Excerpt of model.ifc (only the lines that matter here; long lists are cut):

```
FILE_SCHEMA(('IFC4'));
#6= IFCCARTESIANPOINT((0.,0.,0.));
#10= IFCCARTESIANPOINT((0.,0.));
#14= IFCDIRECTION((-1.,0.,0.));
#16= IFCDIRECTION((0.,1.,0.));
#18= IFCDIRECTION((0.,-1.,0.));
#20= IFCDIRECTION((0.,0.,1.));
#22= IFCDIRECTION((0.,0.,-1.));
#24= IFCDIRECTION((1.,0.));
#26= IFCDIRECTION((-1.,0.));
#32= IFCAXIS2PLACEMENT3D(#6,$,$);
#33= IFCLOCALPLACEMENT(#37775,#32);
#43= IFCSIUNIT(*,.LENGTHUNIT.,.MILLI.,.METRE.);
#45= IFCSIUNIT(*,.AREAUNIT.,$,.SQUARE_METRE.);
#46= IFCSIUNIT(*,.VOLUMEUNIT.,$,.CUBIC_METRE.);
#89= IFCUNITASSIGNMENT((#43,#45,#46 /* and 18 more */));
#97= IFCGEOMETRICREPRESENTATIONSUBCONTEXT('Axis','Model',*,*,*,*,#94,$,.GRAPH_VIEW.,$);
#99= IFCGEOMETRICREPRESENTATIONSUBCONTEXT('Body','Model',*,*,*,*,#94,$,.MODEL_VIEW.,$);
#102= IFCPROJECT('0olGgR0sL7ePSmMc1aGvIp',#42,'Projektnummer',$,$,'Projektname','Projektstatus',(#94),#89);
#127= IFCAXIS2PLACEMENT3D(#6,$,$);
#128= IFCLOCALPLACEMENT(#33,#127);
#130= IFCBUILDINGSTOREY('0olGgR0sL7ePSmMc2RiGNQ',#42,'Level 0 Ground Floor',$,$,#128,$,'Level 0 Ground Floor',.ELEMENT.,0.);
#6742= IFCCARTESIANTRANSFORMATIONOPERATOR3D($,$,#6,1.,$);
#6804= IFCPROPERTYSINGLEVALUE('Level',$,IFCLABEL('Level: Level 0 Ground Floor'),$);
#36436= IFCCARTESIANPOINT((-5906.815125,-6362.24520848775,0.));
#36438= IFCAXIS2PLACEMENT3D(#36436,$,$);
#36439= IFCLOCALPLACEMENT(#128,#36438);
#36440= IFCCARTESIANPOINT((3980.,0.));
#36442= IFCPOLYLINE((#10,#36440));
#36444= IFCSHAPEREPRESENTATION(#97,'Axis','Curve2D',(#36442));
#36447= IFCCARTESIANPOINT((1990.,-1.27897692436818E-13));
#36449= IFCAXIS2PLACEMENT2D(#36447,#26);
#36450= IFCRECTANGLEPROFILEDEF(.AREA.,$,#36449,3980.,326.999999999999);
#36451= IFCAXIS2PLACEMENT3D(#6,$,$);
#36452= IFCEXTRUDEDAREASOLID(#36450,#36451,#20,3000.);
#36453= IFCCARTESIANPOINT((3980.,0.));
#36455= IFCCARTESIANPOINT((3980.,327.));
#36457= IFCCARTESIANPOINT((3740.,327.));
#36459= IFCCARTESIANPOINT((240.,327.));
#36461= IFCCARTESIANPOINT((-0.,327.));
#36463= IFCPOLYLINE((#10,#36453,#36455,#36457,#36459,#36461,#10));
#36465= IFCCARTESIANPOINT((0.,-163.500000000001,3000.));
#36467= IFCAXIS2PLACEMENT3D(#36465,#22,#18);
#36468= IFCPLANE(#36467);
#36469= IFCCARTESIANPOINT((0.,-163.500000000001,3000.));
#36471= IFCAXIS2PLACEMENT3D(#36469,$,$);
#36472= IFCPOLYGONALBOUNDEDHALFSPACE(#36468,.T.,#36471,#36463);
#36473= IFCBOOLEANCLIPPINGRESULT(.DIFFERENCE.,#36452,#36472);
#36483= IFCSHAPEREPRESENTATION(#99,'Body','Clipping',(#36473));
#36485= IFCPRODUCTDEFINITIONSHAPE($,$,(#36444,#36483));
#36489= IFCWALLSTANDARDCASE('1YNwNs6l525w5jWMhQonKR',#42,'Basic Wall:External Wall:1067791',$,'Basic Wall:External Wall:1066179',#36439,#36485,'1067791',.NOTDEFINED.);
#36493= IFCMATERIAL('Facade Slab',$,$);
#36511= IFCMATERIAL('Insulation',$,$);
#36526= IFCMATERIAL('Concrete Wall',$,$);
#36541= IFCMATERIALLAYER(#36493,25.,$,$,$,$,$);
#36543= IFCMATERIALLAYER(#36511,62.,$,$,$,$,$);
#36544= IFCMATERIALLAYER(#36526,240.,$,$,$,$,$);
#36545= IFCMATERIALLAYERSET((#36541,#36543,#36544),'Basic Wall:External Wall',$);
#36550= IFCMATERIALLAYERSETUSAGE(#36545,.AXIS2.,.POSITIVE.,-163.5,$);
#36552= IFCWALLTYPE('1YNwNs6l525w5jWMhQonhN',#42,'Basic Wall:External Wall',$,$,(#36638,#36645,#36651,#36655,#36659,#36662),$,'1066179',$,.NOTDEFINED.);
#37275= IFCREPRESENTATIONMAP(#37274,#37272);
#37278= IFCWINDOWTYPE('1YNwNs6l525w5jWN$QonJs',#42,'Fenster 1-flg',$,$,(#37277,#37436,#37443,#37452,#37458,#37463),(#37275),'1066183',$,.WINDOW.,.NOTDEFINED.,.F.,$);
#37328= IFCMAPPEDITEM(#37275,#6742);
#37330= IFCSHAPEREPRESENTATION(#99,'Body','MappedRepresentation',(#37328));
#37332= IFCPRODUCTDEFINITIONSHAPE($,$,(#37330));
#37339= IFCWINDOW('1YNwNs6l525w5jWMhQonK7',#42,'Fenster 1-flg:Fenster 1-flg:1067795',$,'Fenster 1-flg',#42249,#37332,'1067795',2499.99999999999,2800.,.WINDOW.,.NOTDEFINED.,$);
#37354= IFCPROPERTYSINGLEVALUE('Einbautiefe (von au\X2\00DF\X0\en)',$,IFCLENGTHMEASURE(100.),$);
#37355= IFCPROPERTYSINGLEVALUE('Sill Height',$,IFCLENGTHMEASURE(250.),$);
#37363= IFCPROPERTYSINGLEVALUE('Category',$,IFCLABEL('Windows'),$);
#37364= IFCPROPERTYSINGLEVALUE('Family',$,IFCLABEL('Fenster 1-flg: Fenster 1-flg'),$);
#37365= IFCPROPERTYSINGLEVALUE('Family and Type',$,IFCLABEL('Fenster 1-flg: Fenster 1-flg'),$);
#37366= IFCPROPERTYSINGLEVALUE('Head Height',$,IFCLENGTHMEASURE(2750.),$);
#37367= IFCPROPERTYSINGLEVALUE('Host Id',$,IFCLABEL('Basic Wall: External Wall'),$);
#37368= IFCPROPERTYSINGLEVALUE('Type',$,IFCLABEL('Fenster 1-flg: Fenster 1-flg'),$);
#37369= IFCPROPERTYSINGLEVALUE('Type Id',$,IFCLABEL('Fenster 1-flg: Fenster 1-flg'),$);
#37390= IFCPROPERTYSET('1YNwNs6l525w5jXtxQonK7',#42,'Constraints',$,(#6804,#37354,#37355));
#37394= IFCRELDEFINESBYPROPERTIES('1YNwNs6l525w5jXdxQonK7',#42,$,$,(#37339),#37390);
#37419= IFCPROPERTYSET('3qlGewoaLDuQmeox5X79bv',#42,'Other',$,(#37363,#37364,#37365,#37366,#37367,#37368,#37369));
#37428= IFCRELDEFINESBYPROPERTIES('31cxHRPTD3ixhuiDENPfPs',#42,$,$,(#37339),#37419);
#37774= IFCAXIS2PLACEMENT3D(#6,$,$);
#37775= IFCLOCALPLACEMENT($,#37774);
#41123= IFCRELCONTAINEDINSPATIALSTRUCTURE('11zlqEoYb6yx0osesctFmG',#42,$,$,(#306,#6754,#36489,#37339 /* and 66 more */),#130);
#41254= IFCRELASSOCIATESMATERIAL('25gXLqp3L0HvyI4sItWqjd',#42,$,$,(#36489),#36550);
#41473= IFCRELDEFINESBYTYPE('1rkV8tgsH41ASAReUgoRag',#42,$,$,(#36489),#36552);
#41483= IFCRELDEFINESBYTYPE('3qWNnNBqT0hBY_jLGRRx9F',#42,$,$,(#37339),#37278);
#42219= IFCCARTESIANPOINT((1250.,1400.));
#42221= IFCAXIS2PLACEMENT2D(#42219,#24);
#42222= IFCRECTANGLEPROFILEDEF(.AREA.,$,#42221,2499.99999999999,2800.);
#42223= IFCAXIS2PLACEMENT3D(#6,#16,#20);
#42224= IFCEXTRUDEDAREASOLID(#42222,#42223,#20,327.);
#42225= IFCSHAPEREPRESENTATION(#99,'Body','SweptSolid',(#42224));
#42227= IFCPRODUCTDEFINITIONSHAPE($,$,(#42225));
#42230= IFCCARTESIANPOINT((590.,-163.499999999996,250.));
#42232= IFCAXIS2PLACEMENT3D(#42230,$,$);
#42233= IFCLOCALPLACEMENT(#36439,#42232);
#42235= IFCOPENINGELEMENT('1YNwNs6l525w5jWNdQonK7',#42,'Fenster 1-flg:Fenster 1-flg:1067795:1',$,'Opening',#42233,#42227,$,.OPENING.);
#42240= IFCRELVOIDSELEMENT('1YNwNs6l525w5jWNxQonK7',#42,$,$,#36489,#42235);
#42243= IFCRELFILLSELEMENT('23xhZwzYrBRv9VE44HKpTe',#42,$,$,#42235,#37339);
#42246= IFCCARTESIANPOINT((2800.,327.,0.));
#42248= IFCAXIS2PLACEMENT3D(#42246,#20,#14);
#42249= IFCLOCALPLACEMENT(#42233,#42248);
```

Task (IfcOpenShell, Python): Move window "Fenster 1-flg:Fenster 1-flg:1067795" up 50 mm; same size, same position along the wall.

```python
import numpy as np
import ifcopenshell
import ifcopenshell.api.geometry
import ifcopenshell.api.pset
import ifcopenshell.util.element
import ifcopenshell.util.placement
import ifcopenshell.util.unit

model = ifcopenshell.open("model.ifc")
unit_scale = ifcopenshell.util.unit.calculate_unit_scale(model)

window = model.by_guid("1YNwNs6l525w5jWMhQonK7")
opening = window.FillsVoids[0].RelatingOpeningElement
dz = 0.05 / unit_scale

shift = np.array([0.0, 0.0, dz])
# The window is placed relative to its opening, so it follows when the opening moves.
matrix = ifcopenshell.util.placement.get_local_placement(opening.ObjectPlacement)
matrix[:3, 3] += shift
ifcopenshell.api.geometry.edit_object_placement(
    model, product=opening, matrix=matrix, is_si=False, should_transform_children=True
)

# Keep the stored heights in step.
pset = model.by_id(ifcopenshell.util.element.get_pset(window, "Constraints", should_inherit=False)["id"])
ifcopenshell.api.pset.edit_pset(model, pset=pset, properties={
    "Sill Height": model.create_entity("IfcLengthMeasure", ifcopenshell.util.element.get_pset(window, "Constraints", "Sill Height") + dz),
})
pset = model.by_id(ifcopenshell.util.element.get_pset(window, "Other", should_inherit=False)["id"])
ifcopenshell.api.pset.edit_pset(model, pset=pset, properties={
    "Head Height": model.create_entity("IfcLengthMeasure", ifcopenshell.util.element.get_pset(window, "Other", "Head Height") + dz),
})

print(f"moved by {dz * unit_scale:+.3f} m")

model.write("model_updated.ifc")
```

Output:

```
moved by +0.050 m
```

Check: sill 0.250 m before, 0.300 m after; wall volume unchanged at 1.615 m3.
